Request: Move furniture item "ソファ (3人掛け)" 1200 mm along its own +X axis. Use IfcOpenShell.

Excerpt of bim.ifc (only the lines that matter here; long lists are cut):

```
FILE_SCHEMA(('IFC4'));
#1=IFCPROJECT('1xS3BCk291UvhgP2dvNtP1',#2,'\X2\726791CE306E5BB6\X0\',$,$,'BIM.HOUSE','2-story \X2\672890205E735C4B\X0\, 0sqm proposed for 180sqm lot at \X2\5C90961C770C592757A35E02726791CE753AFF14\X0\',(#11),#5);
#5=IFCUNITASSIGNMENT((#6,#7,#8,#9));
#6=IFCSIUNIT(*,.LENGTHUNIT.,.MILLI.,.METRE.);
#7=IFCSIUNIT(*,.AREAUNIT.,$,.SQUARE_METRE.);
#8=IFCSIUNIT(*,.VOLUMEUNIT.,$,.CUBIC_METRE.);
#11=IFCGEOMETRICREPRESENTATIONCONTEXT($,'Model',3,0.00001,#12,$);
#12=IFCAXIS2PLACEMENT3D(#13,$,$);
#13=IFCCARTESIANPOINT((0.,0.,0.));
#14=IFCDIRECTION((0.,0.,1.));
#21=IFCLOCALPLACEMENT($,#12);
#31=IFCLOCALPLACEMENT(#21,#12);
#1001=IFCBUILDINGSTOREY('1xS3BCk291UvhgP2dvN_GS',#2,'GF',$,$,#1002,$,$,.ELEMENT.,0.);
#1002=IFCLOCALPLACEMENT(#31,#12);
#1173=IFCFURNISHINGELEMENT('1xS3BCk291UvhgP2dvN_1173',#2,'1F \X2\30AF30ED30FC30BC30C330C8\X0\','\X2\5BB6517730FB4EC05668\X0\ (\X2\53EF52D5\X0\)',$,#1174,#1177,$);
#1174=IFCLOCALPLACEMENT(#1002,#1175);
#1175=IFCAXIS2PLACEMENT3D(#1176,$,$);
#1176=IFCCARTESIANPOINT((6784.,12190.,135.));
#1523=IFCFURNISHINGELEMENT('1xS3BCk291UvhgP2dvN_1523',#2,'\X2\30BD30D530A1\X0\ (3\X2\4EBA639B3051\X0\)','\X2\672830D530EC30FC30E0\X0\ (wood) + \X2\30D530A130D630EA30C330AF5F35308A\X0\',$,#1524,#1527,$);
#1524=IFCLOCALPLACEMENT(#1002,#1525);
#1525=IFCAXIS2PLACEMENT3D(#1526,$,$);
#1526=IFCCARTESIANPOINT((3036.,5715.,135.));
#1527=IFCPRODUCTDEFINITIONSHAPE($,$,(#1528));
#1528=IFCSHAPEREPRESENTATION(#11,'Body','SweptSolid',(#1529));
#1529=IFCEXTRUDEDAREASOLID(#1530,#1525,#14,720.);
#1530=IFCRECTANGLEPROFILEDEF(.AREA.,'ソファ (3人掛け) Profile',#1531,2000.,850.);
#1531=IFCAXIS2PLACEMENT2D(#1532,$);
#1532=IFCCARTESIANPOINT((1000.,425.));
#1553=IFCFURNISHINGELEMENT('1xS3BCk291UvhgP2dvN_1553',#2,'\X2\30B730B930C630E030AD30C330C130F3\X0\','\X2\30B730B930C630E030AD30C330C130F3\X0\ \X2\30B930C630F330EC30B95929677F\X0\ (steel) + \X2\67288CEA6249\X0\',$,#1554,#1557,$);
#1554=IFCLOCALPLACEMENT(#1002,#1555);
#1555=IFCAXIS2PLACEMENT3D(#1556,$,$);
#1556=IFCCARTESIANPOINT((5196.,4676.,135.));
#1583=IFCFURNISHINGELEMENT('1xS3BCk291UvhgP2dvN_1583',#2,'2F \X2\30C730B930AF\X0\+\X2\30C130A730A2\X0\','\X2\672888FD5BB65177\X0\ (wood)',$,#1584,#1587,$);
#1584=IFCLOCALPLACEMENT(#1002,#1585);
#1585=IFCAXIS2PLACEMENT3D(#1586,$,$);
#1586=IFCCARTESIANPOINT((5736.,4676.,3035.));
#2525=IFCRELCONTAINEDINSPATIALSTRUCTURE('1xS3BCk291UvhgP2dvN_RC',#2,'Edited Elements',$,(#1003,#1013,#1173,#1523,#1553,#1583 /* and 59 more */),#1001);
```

```python
import ifcopenshell
import ifcopenshell.api.geometry
import ifcopenshell.util.placement
import ifcopenshell.util.unit

model = ifcopenshell.open("bim.ifc")
unit_scale = ifcopenshell.util.unit.calculate_unit_scale(model)

item = model.by_guid("1xS3BCk291UvhgP2dvN_1523")
matrix = ifcopenshell.util.placement.get_local_placement(item.ObjectPlacement)
matrix[:3, 3] += matrix[:3, 0] * 1.2 / unit_scale
ifcopenshell.api.geometry.edit_object_placement(model, product=item, matrix=matrix, is_si=False)

print(ifcopenshell.util.placement.get_local_placement(item.ObjectPlacement).round(3) + 0.0)

model.write("bim_rev.ifc")
```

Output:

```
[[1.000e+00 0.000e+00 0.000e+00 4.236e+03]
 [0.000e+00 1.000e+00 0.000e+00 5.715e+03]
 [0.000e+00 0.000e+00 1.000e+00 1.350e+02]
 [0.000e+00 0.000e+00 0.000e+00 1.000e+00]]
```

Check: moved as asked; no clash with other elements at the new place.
